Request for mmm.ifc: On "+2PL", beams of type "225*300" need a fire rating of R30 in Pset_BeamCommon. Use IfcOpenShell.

First a look at what the model holds.

```python
import ifcopenshell
import ifcopenshell.util.element

model = ifcopenshell.open("mmm.ifc")
print(model.schema)
storey = next(s for s in model.by_type("IfcBuildingStorey") if s.Name == "+2PL")
beams = [e for e in ifcopenshell.util.element.get_decomposition(storey) if e.is_a("IfcBeam")]
seen = {}
for e in beams:
    element_type = ifcopenshell.util.element.get_type(e)
    key = (element_type.Name if element_type != e and element_type else None, ifcopenshell.util.element.get_pset(e, "Pset_BeamCommon", "FireRating"))
    seen[key] = seen.get(key, 0) + 1
for (name, value), count in sorted(seen.items(), key=str):
    print(count, "x", name, "|", value)
```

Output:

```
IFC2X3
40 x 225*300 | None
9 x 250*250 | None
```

```python
import ifcopenshell
import ifcopenshell.api.pset
import ifcopenshell.util.element

model = ifcopenshell.open("mmm.ifc")

storey = next(s for s in model.by_type("IfcBuildingStorey") if s.Name == "+2PL")
beams = [e for e in ifcopenshell.util.element.get_decomposition(storey) if e.is_a("IfcBeam")]

count = 0
for e in beams:
    element_type = ifcopenshell.util.element.get_type(e)
    if element_type in (None, e) or element_type.Name != "225*300":
        continue
    found = ifcopenshell.util.element.get_pset(e, "Pset_BeamCommon", should_inherit=False)
    if found:
        pset = model.by_id(found["id"])
        if len(ifcopenshell.util.element.get_elements_by_pset(pset)) > 1:
            pset = ifcopenshell.api.pset.unshare_pset(model, products=[e], pset=pset)[0]
    else:
        pset = ifcopenshell.api.pset.add_pset(model, product=e, name="Pset_BeamCommon")
    ifcopenshell.api.pset.edit_pset(model, pset=pset, properties={"FireRating": "R30"})
    count += 1

print(count, "beams updated")

model.write("mmm_updated.ifc")
```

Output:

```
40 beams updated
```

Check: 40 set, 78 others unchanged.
